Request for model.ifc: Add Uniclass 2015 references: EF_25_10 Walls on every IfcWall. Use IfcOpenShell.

First a look at what the model holds.

```python
import ifcopenshell

model = ifcopenshell.open("model.ifc")
print(model.schema)
print("classifications:", [c.Name for c in model.by_type("IfcClassification")])
for ifc_class in ("IfcDoor", "IfcRoof", "IfcStair", "IfcWall", "IfcWindow"):
    print(ifc_class, len(model.by_type(ifc_class)))
```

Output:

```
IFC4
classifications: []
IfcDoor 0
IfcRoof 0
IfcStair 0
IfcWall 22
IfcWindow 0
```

```python
import ifcopenshell
import ifcopenshell.api.classification

model = ifcopenshell.open("model.ifc")

system = ifcopenshell.api.classification.add_classification(model, classification="Uniclass 2015")

codes = {
    "IfcWall": ("EF_25_10", "Walls"),
}
for ifc_class, (code, name) in codes.items():
    products = model.by_type(ifc_class)
    ifcopenshell.api.classification.add_reference(
        model, products=products, classification=system, identification=code, name=name
    )
    print(code, len(products))

model.write("model_v2.ifc")
```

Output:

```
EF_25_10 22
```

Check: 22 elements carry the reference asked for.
